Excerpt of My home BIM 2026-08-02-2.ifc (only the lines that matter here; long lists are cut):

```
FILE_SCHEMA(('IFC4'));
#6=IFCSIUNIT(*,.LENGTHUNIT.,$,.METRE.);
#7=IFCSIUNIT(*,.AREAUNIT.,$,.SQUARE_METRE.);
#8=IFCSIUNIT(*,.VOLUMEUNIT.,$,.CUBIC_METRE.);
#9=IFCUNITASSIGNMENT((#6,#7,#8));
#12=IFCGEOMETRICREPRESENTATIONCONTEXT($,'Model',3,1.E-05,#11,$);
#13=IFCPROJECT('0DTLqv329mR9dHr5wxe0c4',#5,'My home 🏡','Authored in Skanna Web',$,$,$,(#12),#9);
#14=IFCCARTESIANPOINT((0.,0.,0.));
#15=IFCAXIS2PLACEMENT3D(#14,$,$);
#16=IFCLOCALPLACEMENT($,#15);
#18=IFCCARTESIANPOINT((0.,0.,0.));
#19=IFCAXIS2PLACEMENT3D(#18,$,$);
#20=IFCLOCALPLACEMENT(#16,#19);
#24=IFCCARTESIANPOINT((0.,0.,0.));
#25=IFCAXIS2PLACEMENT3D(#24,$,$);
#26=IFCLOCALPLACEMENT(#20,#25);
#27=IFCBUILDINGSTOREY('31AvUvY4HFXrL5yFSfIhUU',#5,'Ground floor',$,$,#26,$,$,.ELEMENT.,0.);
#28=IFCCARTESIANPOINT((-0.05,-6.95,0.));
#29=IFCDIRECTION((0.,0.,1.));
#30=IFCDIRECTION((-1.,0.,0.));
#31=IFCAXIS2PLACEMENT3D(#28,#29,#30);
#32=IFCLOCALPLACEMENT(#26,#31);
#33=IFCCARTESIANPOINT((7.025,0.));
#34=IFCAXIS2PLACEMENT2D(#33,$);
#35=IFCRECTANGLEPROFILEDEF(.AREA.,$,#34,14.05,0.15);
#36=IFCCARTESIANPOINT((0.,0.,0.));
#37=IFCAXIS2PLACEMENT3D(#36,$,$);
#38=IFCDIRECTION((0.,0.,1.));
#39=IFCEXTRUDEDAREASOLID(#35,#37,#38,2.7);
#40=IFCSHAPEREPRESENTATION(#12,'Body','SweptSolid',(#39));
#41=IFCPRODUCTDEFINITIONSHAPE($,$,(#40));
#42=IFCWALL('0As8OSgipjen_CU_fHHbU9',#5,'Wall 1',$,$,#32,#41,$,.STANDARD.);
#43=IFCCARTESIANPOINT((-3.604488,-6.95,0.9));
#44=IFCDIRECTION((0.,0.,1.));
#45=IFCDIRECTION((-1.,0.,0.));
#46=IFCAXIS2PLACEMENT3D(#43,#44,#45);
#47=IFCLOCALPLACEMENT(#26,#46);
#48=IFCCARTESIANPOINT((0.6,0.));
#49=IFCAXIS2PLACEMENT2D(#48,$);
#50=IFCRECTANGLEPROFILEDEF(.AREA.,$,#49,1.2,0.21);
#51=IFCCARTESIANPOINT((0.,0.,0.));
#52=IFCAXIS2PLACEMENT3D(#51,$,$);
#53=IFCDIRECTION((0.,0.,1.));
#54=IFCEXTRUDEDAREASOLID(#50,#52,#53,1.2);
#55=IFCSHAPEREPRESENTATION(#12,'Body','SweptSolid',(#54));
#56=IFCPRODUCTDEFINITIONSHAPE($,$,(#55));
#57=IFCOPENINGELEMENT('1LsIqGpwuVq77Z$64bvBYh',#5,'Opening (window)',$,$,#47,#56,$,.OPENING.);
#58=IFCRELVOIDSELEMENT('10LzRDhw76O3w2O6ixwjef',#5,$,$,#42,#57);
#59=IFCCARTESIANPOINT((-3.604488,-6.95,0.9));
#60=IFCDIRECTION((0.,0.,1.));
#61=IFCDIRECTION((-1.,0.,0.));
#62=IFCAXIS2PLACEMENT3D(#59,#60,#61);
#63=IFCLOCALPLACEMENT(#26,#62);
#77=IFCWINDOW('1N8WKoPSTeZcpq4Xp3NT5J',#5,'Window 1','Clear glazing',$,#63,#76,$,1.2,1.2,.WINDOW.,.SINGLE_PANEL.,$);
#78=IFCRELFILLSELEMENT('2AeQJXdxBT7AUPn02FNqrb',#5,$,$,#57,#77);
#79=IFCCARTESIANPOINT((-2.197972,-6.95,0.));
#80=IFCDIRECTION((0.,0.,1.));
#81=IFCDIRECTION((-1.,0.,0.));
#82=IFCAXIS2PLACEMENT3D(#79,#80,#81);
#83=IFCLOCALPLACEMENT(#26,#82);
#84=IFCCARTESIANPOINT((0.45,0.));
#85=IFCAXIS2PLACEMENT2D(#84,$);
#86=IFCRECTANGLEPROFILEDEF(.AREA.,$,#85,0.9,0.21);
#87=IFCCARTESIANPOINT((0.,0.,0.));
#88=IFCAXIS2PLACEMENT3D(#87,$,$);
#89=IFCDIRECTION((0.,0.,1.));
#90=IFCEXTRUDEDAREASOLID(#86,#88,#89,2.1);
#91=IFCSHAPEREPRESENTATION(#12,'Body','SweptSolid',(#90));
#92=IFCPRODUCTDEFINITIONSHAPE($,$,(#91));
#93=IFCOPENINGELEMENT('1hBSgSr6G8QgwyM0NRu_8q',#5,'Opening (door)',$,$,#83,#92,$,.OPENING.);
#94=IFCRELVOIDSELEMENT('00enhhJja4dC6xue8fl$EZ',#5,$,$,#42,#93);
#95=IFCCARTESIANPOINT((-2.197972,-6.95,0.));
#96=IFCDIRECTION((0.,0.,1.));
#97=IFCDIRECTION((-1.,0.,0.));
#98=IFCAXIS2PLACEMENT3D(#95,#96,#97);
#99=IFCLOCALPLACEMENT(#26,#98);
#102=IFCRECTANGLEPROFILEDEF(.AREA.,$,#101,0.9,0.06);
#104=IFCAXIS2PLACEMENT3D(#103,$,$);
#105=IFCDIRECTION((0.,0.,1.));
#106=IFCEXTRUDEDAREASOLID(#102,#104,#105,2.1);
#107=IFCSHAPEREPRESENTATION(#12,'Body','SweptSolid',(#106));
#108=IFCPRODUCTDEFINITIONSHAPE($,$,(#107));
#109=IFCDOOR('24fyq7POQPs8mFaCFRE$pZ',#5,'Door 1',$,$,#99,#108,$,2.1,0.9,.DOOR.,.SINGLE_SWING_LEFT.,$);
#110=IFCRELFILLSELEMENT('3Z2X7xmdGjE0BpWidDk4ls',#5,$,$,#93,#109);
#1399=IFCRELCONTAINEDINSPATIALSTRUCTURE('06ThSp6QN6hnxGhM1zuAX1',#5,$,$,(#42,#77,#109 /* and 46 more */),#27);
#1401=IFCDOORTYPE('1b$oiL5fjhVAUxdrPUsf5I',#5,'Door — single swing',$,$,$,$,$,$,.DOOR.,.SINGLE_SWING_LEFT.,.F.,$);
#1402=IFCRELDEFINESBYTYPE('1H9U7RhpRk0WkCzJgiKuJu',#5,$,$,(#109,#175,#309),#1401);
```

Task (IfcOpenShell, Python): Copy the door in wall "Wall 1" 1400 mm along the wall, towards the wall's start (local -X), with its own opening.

```python
import ifcopenshell
import ifcopenshell.api.feature
import ifcopenshell.api.geometry
import ifcopenshell.api.root
import ifcopenshell.geom
import ifcopenshell.util.element
import ifcopenshell.util.placement
import ifcopenshell.util.shape
import ifcopenshell.util.unit

model = ifcopenshell.open("My home BIM 2026-08-02-2.ifc")
unit_scale = ifcopenshell.util.unit.calculate_unit_scale(model)
settings = ifcopenshell.geom.settings()


def volume(element):
    """Net volume in cubic metres, openings subtracted."""
    shape = ifcopenshell.geom.create_shape(settings, element)
    return ifcopenshell.util.shape.get_volume(shape.geometry)


door = model.by_guid("24fyq7POQPs8mFaCFRE$pZ")
opening = door.FillsVoids[0].RelatingOpeningElement
wall = opening.VoidsElements[0].RelatingBuildingElement
before = volume(wall)
shift = ifcopenshell.util.placement.get_local_placement(wall.ObjectPlacement)[:3, 0] * -1.4 / unit_scale

# copy_class copies the void relationship, type, container and properties, but no geometry.
new_opening = ifcopenshell.api.root.copy_class(model, product=opening)
new_opening.Representation = ifcopenshell.util.element.copy_deep(
    model, opening.Representation, exclude=["IfcGeometricRepresentationContext", "IfcRepresentationMap"]
)
new_door = ifcopenshell.api.root.copy_class(model, product=door)
new_door.Representation = ifcopenshell.util.element.copy_deep(
    model, door.Representation, exclude=["IfcGeometricRepresentationContext", "IfcRepresentationMap"]
)
ifcopenshell.api.feature.add_filling(model, opening=new_opening, element=new_door)

for old, new in ((opening, new_opening), (door, new_door)):
    matrix = ifcopenshell.util.placement.get_local_placement(old.ObjectPlacement)
    matrix[:3, 3] += shift
    ifcopenshell.api.geometry.edit_object_placement(model, product=new, matrix=matrix, is_si=False)

after = volume(wall)

print(f"wall volume {before:.3f} -> {after:.3f} m3")

model.write("My home BIM 2026-08-02-2-out.ifc")
```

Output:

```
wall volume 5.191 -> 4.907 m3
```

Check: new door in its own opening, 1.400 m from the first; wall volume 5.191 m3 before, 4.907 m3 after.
